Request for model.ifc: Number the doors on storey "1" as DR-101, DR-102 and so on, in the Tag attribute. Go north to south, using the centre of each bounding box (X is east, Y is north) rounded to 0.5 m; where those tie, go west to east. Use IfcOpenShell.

First a look at what the model holds.

```python
import ifcopenshell
import ifcopenshell.util.element
import ifcopenshell.util.placement

model = ifcopenshell.open("model.ifc")
print(model.schema)
storey = next(s for s in model.by_type("IfcBuildingStorey") if s.Name == "1")
doors = [e for e in ifcopenshell.util.element.get_decomposition(storey) if e.is_a("IfcDoor")]
for e in sorted(doors, key=lambda e: e.id()):
    origin = ifcopenshell.util.placement.get_local_placement(e.ObjectPlacement)[:3, 3]
    print(e.id(), e.Tag, e.Name, origin.round(2) + 0.0, sep=" | ")
```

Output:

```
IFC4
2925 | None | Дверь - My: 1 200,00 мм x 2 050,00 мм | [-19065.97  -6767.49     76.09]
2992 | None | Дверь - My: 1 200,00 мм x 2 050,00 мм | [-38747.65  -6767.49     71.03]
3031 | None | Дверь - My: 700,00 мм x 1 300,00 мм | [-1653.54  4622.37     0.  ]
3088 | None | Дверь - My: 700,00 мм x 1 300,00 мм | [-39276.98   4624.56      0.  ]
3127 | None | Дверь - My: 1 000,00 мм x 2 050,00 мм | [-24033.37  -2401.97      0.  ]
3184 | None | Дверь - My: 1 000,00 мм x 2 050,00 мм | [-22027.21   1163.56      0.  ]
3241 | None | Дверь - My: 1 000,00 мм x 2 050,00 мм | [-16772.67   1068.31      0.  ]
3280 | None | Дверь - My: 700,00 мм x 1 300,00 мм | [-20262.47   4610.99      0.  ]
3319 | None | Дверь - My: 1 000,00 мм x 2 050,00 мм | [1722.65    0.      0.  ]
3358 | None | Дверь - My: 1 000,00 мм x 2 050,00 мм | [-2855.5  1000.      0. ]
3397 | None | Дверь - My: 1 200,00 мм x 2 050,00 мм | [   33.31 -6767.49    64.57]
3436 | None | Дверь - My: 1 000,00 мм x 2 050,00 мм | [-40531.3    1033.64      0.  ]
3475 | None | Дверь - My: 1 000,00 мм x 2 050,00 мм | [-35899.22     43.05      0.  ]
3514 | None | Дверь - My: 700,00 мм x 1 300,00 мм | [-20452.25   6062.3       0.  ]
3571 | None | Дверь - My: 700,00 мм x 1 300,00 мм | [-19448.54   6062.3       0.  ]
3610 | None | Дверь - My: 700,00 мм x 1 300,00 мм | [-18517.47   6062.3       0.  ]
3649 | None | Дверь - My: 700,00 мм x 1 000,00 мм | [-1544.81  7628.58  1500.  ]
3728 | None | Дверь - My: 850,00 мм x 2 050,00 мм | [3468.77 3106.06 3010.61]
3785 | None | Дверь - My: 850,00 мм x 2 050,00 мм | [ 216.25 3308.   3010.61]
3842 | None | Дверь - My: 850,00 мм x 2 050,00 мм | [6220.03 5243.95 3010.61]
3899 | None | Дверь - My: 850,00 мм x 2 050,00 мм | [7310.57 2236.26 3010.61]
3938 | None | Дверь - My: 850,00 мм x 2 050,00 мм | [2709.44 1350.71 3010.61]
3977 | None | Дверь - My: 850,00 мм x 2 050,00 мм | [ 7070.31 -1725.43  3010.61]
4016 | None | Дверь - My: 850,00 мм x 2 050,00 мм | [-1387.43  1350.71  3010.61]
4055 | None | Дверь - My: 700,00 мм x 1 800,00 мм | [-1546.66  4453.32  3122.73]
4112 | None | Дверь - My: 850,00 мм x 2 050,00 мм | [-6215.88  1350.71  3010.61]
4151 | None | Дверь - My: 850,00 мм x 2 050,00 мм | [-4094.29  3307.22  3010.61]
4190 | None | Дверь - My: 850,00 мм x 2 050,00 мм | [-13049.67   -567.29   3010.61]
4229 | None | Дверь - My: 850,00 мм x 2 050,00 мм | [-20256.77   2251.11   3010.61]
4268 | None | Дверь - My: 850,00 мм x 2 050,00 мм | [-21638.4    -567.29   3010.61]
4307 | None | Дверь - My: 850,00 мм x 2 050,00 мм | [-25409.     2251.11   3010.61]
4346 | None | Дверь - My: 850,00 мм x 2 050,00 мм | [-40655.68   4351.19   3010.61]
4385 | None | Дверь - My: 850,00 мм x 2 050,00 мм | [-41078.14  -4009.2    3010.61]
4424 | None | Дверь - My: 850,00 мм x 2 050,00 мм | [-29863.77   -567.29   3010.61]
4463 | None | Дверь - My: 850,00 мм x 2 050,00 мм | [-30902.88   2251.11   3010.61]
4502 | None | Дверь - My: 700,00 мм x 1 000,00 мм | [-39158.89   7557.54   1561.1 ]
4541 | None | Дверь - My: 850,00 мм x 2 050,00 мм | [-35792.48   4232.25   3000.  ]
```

```python
import ifcopenshell
import ifcopenshell.geom
import ifcopenshell.util.element
import ifcopenshell.util.shape

model = ifcopenshell.open("model.ifc")
settings = ifcopenshell.geom.settings()
settings.set("use-world-coords", True)


def centre(element):
    shape = ifcopenshell.geom.create_shape(settings, element)
    return ifcopenshell.util.shape.get_bbox_centroid(shape.geometry)


storey = next(s for s in model.by_type("IfcBuildingStorey") if s.Name == "1")
doors = [e for e in ifcopenshell.util.element.get_decomposition(storey) if e.is_a("IfcDoor")]

# Insertion points can sit at a corner or the storey origin, so sort by the geometry (in metres).
centres = {e: centre(e) for e in doors}
doors.sort(key=lambda e: (-round(centres[e][1] / 0.5), centres[e][0]))

for i, e in enumerate(doors, start=1):
    number = f"DR-1{i:02d}"
    e.Tag = number
    print(e.id(), number)

model.write("model_edited.ifc")
```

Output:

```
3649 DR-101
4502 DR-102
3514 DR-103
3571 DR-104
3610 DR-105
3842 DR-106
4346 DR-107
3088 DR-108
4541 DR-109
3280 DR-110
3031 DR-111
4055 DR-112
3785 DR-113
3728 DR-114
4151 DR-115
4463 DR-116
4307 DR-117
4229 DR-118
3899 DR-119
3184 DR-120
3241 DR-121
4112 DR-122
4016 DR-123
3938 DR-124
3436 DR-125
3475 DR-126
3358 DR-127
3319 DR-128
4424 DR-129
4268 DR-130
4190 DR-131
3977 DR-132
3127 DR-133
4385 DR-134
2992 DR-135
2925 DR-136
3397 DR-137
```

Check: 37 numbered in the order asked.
